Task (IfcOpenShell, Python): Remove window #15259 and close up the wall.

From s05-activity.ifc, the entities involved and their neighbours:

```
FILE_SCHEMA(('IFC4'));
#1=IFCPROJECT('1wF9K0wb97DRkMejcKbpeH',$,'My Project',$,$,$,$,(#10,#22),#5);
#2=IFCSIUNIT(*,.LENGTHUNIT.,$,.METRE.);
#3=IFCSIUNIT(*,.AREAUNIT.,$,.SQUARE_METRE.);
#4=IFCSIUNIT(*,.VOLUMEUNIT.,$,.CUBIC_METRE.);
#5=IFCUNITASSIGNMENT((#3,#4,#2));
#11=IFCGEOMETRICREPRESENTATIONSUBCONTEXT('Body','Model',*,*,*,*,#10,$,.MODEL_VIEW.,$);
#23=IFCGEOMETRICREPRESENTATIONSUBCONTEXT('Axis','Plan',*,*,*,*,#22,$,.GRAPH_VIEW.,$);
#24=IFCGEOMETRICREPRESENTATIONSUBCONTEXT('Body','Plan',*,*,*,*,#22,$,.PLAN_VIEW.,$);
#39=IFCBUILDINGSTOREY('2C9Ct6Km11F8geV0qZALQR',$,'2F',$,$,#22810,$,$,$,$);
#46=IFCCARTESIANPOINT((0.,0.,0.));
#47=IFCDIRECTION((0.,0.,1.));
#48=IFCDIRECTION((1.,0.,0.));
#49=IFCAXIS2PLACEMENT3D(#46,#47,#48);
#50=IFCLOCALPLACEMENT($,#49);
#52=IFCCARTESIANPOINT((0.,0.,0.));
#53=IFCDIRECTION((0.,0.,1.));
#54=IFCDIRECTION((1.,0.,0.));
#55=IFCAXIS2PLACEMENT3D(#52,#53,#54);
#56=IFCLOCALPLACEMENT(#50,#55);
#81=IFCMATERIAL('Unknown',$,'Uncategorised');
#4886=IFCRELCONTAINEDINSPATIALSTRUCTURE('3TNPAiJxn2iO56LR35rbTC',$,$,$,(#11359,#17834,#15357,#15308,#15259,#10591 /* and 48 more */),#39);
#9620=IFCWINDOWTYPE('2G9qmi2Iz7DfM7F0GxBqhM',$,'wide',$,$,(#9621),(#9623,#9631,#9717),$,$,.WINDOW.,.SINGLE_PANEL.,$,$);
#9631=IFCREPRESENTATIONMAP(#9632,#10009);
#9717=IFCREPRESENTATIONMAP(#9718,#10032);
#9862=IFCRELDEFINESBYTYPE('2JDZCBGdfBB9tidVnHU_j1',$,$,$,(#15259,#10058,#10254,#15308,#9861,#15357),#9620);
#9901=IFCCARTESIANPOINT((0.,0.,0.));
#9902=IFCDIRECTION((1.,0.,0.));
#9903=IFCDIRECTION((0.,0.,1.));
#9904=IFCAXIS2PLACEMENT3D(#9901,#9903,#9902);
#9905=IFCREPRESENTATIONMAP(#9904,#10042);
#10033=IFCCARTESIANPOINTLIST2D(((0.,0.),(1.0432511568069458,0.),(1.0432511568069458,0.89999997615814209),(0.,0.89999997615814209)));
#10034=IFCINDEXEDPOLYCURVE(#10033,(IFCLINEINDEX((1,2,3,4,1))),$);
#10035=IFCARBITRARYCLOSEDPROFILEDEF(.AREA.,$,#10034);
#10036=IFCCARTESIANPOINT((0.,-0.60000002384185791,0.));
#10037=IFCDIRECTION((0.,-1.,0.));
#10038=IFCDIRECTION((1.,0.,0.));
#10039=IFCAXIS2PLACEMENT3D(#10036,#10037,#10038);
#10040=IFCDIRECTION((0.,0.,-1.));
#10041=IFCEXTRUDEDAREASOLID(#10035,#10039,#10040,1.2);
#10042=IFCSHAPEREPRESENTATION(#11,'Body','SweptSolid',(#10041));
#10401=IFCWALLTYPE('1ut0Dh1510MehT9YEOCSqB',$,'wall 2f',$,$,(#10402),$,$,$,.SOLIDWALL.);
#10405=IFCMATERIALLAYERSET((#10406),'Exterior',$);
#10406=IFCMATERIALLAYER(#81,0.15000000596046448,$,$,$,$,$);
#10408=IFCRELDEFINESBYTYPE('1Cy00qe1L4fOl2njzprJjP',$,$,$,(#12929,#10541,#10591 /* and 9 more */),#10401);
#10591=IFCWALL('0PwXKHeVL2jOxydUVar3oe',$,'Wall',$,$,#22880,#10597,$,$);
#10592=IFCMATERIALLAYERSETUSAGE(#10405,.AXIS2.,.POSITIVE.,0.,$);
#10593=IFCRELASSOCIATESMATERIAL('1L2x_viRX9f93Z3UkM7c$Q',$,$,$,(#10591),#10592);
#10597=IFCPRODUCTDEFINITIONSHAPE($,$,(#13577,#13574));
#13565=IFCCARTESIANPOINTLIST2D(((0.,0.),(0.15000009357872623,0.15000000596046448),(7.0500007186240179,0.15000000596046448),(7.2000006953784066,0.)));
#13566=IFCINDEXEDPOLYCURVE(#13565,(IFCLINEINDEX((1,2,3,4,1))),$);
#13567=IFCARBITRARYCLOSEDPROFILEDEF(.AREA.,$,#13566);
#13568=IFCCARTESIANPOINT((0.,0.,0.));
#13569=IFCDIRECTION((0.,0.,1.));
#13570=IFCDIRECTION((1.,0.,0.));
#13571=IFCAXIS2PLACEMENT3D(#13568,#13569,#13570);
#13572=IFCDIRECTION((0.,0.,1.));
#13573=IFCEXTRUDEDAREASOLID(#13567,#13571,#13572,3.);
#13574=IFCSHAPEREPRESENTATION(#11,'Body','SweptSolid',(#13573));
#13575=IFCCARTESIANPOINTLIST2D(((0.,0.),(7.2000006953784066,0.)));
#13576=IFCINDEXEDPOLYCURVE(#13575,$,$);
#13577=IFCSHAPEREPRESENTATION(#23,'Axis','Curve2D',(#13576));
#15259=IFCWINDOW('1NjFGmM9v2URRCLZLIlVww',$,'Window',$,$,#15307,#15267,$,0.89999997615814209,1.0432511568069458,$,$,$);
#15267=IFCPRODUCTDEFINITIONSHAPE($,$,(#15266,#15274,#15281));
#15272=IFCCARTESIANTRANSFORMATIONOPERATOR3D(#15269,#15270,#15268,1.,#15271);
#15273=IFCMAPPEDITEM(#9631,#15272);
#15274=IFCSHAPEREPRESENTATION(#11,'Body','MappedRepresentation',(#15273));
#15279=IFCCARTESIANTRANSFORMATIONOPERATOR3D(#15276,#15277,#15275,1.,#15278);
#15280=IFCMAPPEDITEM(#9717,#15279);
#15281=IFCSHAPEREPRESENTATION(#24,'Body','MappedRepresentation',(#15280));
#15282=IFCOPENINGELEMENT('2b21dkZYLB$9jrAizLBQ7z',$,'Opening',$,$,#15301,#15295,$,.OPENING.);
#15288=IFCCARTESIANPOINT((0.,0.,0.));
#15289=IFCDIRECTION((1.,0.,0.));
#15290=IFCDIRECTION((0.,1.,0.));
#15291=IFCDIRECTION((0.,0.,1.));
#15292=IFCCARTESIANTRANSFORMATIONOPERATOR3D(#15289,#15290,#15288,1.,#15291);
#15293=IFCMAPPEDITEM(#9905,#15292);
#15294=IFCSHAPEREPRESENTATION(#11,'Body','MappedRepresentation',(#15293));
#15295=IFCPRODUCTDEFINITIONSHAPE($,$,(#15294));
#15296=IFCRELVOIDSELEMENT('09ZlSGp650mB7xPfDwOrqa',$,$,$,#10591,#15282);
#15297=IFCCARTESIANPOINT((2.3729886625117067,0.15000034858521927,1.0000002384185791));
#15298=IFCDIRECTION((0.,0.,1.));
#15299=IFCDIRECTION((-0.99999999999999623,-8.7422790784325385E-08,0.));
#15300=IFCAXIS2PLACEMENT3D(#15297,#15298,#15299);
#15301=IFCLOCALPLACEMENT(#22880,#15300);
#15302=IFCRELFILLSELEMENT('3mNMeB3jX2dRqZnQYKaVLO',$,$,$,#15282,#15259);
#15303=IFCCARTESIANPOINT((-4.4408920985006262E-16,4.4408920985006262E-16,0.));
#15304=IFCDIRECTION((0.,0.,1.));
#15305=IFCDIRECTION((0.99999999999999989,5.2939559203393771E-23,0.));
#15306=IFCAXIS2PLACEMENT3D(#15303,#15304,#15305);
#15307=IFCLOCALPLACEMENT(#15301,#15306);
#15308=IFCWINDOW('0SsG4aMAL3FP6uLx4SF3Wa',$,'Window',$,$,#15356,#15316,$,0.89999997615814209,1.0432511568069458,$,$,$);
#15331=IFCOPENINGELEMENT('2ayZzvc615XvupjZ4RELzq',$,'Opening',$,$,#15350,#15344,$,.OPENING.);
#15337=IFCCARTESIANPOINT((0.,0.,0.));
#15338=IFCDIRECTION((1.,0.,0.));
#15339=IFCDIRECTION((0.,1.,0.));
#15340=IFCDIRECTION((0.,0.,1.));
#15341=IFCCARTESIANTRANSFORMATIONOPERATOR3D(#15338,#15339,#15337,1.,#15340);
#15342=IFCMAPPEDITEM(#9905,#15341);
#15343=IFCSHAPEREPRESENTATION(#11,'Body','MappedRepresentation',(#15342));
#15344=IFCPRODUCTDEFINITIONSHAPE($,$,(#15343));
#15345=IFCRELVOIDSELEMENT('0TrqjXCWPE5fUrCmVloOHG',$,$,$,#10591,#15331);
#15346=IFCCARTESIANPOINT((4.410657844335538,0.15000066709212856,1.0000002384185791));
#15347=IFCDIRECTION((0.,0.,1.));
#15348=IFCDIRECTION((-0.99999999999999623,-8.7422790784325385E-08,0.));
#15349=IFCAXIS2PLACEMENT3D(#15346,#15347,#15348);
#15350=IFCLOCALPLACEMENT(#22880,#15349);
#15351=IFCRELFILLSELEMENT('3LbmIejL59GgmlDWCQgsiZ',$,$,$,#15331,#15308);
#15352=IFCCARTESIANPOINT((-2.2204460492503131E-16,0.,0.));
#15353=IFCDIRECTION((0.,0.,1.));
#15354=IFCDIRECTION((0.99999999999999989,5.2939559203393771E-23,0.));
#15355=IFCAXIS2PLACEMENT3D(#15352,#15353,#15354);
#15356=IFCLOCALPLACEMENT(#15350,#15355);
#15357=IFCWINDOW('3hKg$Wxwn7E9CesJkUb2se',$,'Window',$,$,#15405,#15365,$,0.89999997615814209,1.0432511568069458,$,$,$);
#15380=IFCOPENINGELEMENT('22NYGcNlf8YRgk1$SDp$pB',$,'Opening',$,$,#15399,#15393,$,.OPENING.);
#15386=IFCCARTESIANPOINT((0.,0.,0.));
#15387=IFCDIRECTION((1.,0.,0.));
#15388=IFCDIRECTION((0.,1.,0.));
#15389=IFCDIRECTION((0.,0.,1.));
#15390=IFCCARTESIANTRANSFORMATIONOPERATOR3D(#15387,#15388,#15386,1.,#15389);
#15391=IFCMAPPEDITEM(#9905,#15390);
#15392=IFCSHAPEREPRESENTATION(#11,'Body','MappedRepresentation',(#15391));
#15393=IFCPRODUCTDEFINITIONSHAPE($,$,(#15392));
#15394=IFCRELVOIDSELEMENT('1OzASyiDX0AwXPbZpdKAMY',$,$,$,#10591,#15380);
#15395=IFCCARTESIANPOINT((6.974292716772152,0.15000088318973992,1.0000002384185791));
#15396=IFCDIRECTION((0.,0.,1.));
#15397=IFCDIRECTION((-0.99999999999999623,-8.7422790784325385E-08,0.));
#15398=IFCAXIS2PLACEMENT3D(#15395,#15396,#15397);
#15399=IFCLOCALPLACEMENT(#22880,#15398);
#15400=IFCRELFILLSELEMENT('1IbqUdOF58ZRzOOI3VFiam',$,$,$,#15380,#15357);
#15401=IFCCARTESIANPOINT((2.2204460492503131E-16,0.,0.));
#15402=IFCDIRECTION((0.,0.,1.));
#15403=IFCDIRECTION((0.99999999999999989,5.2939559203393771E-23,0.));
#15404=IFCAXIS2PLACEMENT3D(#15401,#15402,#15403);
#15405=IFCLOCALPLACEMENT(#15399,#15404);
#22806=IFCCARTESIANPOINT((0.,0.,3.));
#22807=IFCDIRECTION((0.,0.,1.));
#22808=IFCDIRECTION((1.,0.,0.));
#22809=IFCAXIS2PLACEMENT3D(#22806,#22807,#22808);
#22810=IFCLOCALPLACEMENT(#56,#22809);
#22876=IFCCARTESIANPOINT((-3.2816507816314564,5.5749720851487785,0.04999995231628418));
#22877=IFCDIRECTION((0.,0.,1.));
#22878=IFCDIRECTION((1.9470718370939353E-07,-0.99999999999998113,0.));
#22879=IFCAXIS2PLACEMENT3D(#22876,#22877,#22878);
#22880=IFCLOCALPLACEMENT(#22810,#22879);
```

```python
import ifcopenshell
import ifcopenshell.api.feature
import ifcopenshell.api.root
import ifcopenshell.geom
import ifcopenshell.util.shape

model = ifcopenshell.open("s05-activity.ifc")
settings = ifcopenshell.geom.settings()


def volume(element):
    """Net volume in cubic metres, openings subtracted."""
    shape = ifcopenshell.geom.create_shape(settings, element)
    return ifcopenshell.util.shape.get_volume(shape.geometry)


window = model.by_guid("1NjFGmM9v2URRCLZLIlVww")
opening = window.FillsVoids[0].RelatingOpeningElement
wall = opening.VoidsElements[0].RelatingBuildingElement
before = volume(wall)

ifcopenshell.api.root.remove_product(model, product=window)
ifcopenshell.api.feature.remove_feature(model, feature=opening)

after = volume(wall)

print(f"wall volume {before:.3f} -> {after:.3f} m3")

model.write("s05-activity_rev.ifc")
```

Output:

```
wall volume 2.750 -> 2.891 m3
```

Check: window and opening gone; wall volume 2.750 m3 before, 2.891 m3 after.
